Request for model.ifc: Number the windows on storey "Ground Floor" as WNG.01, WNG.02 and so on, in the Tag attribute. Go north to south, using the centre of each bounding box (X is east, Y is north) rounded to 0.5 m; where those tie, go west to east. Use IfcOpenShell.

First a look at what the model holds.

```python
import ifcopenshell
import ifcopenshell.util.element
import ifcopenshell.util.placement

model = ifcopenshell.open("model.ifc")
print(model.schema)
storey = next(s for s in model.by_type("IfcBuildingStorey") if s.Name == "Ground Floor")
windows = [e for e in ifcopenshell.util.element.get_decomposition(storey) if e.is_a("IfcWindow")]
for e in sorted(windows, key=lambda e: e.id()):
    origin = ifcopenshell.util.placement.get_local_placement(e.ObjectPlacement)[:3, 3]
    print(e.id(), e.Tag, e.Name, origin.round(2) + 0.0, sep=" | ")
```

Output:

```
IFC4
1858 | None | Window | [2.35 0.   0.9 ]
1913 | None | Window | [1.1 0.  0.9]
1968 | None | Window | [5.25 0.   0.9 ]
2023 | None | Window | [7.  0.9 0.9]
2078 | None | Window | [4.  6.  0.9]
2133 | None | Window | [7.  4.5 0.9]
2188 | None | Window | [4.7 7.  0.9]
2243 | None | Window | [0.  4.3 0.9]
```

```python
import ifcopenshell
import ifcopenshell.geom
import ifcopenshell.util.element
import ifcopenshell.util.shape

model = ifcopenshell.open("model.ifc")
settings = ifcopenshell.geom.settings()
settings.set("use-world-coords", True)


def centre(element):
    shape = ifcopenshell.geom.create_shape(settings, element)
    return ifcopenshell.util.shape.get_bbox_centroid(shape.geometry)


storey = next(s for s in model.by_type("IfcBuildingStorey") if s.Name == "Ground Floor")
windows = [e for e in ifcopenshell.util.element.get_decomposition(storey) if e.is_a("IfcWindow")]

# Insertion points can sit at a corner or the storey origin, so sort by the geometry (in metres).
centres = {e: centre(e) for e in windows}
windows.sort(key=lambda e: (-round(centres[e][1] / 0.5), centres[e][0]))

for i, e in enumerate(windows, start=1):
    number = f"WNG.{i:02d}"
    e.Tag = number
    print(e.id(), number)

model.write("model_v2.ifc")
```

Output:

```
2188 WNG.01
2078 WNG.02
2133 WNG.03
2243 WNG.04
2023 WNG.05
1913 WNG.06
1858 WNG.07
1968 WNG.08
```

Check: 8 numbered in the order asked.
